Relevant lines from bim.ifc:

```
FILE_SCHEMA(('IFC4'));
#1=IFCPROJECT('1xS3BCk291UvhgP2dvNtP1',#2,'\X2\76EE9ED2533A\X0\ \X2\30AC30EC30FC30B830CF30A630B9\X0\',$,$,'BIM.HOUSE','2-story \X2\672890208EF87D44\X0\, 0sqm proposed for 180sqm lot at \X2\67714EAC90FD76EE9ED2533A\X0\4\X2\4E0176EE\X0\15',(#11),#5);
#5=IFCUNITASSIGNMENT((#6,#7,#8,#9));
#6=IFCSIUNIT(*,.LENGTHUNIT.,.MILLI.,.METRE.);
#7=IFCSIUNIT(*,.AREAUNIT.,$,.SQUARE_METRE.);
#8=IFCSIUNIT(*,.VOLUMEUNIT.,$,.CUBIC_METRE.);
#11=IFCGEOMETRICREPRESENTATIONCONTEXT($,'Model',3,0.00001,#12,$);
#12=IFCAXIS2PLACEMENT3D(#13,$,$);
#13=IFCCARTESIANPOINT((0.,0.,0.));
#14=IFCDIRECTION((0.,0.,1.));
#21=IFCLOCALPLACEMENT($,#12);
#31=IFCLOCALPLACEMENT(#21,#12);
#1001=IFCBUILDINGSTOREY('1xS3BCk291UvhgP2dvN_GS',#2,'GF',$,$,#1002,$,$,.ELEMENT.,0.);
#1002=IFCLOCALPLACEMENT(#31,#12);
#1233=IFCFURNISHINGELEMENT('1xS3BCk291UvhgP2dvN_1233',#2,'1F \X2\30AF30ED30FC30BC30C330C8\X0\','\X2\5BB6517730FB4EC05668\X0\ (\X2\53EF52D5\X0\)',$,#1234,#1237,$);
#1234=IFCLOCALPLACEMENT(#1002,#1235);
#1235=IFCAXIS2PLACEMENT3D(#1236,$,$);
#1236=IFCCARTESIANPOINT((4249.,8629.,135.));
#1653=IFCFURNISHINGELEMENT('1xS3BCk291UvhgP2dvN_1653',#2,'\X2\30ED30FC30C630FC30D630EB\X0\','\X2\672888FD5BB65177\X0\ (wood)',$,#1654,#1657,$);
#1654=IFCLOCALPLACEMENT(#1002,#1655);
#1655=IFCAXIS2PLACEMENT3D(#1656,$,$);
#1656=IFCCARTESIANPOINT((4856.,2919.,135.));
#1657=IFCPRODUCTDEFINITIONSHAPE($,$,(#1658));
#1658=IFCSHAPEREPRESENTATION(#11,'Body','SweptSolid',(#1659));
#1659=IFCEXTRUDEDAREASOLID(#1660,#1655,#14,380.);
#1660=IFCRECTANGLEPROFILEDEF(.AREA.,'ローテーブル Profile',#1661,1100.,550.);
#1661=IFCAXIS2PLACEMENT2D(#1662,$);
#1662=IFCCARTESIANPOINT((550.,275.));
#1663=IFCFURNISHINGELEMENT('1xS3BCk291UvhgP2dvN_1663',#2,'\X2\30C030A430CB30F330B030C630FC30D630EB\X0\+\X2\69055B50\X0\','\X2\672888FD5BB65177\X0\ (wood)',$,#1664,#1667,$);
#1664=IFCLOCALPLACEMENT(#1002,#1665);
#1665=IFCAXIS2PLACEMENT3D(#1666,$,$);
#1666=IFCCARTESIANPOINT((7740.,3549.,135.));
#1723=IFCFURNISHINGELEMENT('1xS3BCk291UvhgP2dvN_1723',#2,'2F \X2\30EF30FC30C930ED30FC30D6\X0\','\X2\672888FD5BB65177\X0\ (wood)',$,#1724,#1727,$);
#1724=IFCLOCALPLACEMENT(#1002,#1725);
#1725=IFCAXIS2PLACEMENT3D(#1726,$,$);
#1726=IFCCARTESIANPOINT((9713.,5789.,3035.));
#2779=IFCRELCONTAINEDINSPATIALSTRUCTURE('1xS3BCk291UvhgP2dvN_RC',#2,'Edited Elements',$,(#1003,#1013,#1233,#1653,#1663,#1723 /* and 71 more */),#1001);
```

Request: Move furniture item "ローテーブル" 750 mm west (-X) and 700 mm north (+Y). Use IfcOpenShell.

```python
import ifcopenshell
import ifcopenshell.api.geometry
import ifcopenshell.util.placement
import ifcopenshell.util.unit

model = ifcopenshell.open("bim.ifc")
unit_scale = ifcopenshell.util.unit.calculate_unit_scale(model)

item = model.by_id(1653)
matrix = ifcopenshell.util.placement.get_local_placement(item.ObjectPlacement)
matrix[0, 3] -= 0.75 / unit_scale
matrix[1, 3] += 0.7 / unit_scale
ifcopenshell.api.geometry.edit_object_placement(model, product=item, matrix=matrix, is_si=False)

print(ifcopenshell.util.placement.get_local_placement(item.ObjectPlacement).round(3) + 0.0)

model.write("bim_v2.ifc")
```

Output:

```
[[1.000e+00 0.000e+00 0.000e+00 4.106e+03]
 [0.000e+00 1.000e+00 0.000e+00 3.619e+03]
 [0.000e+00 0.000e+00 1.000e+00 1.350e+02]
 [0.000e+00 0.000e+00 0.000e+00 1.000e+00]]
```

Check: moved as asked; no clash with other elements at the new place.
